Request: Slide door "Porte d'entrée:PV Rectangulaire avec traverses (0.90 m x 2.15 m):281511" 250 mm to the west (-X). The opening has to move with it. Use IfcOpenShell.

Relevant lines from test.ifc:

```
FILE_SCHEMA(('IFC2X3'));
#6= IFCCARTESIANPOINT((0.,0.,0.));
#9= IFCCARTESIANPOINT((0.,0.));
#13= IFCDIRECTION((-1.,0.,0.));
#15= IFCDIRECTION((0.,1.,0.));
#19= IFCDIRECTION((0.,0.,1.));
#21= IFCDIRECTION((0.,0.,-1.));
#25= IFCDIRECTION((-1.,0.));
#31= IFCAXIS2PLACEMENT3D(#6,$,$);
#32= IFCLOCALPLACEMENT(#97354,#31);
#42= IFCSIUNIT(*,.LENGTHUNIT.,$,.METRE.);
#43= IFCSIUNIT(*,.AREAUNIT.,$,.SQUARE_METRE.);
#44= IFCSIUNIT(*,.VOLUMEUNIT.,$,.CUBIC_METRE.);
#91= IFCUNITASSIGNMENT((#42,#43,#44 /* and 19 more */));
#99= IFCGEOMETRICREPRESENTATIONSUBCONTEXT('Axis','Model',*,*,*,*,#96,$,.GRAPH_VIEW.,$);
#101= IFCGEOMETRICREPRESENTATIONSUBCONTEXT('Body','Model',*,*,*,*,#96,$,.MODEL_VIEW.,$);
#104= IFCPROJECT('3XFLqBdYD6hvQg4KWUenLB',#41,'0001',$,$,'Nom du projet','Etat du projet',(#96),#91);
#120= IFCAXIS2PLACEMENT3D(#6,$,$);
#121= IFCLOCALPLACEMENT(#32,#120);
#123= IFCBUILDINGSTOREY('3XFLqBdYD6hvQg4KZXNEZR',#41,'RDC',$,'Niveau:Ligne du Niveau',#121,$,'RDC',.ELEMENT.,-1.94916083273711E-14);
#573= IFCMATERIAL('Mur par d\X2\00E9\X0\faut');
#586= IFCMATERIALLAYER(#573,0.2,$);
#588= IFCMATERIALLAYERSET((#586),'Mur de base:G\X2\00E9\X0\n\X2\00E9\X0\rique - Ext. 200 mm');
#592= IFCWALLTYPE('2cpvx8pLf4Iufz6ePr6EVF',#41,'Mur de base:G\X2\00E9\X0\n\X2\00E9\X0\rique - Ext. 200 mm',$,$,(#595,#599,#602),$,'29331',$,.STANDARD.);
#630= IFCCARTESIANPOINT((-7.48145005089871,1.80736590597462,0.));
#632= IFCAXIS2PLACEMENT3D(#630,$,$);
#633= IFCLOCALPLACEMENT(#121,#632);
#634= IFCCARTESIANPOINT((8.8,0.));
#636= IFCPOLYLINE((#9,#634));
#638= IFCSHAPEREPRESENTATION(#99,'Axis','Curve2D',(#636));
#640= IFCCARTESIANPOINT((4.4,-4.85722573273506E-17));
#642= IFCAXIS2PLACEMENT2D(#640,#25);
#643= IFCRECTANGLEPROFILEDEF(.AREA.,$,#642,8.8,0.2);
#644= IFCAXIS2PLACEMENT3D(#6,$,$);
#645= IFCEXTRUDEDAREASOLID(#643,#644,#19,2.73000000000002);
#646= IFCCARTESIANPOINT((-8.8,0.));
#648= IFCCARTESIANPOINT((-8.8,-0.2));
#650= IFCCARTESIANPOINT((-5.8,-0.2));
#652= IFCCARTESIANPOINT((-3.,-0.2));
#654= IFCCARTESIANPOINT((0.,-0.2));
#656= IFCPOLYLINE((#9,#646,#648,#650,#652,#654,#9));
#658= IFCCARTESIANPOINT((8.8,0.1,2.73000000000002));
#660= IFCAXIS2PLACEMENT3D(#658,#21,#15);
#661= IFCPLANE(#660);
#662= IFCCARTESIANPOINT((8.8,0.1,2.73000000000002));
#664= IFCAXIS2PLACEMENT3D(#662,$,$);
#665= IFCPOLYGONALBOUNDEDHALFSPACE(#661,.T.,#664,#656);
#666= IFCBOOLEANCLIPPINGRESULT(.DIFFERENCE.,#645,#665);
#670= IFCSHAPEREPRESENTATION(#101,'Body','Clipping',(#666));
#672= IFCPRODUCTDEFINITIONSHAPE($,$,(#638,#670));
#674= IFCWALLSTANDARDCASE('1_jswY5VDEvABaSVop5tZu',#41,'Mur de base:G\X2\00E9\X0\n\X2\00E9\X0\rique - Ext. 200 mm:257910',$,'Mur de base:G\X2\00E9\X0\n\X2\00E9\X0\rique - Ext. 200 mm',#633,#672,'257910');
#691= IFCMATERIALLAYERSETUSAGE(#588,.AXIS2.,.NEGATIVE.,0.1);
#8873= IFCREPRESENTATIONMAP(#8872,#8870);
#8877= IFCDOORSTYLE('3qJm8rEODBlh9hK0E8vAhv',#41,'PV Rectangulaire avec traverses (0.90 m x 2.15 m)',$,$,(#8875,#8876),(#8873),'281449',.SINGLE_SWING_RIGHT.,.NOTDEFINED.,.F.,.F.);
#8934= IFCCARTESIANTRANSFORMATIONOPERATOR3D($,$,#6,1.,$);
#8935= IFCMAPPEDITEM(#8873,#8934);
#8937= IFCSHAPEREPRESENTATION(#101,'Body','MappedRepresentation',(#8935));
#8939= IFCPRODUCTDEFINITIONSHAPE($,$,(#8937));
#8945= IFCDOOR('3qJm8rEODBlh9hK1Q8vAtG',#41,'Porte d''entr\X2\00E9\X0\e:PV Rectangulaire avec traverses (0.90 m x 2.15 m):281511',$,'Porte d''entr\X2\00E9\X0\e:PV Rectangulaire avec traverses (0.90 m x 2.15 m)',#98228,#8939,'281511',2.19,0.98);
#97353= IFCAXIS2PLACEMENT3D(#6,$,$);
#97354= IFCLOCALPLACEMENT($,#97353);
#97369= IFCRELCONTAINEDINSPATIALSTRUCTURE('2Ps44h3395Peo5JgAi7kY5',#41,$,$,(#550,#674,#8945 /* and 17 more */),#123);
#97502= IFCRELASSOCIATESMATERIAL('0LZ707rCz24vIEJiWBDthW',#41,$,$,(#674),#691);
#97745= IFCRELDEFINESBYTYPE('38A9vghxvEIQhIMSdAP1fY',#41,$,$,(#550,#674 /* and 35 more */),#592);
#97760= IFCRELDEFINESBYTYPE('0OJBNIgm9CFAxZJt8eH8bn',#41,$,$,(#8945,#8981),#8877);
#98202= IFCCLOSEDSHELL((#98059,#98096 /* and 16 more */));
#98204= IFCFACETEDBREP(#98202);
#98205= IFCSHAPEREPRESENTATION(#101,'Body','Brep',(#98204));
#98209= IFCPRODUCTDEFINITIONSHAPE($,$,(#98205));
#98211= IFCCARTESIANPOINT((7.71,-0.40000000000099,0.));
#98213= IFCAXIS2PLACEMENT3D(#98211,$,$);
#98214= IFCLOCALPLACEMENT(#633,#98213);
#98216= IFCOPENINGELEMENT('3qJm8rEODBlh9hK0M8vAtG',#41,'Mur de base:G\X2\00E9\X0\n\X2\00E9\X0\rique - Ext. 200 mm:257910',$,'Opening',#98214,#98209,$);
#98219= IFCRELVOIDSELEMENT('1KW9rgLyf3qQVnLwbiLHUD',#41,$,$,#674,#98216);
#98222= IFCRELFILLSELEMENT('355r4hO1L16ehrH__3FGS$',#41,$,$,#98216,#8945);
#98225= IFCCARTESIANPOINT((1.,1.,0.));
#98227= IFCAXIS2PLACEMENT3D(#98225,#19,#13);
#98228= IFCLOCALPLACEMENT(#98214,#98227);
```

```python
import ifcopenshell
import ifcopenshell.api.geometry
import ifcopenshell.util.placement

model = ifcopenshell.open("test.ifc")

door = model.by_guid("3qJm8rEODBlh9hK1Q8vAtG")
opening = door.FillsVoids[0].RelatingOpeningElement
wall = opening.VoidsElements[0].RelatingBuildingElement

wall_matrix = ifcopenshell.util.placement.get_local_placement(wall.ObjectPlacement)
shift = wall_matrix[:3, 0] * -0.25
before = ifcopenshell.util.placement.get_local_placement(door.ObjectPlacement)[:3, 3].copy()

# The door is placed relative to its opening, so it follows when the opening moves.
matrix = ifcopenshell.util.placement.get_local_placement(opening.ObjectPlacement)
matrix[:3, 3] += shift
ifcopenshell.api.geometry.edit_object_placement(
    model, product=opening, matrix=matrix, is_si=False, should_transform_children=True
)

after = ifcopenshell.util.placement.get_local_placement(door.ObjectPlacement)[:3, 3]
print("door moved by", (after - before).round(3) + 0.0)

model.write("test_updated.ifc")
```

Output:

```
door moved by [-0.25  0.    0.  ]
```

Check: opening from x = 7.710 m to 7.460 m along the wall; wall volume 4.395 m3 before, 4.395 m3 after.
